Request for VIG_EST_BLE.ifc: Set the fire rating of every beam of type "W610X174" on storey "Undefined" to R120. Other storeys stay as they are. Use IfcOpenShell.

First a look at what the model holds.

```python
import ifcopenshell
import ifcopenshell.util.element

model = ifcopenshell.open("VIG_EST_BLE.ifc")
print(model.schema)
storey = next(s for s in model.by_type("IfcBuildingStorey") if s.Name == "Undefined")
beams = [e for e in ifcopenshell.util.element.get_decomposition(storey) if e.is_a("IfcBeam")]
seen = {}
for e in beams:
    element_type = ifcopenshell.util.element.get_type(e)
    key = (element_type.Name if element_type != e and element_type else None, ifcopenshell.util.element.get_pset(e, "Pset_BeamCommon", "FireRating"))
    seen[key] = seen.get(key, 0) + 1
for (name, value), count in sorted(seen.items(), key=str):
    print(count, "x", name, "|", value)
```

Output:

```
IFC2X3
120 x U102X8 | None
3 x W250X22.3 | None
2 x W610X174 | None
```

```python
import ifcopenshell
import ifcopenshell.api.pset
import ifcopenshell.util.element

model = ifcopenshell.open("VIG_EST_BLE.ifc")

storey = next(s for s in model.by_type("IfcBuildingStorey") if s.Name == "Undefined")
beams = [e for e in ifcopenshell.util.element.get_decomposition(storey) if e.is_a("IfcBeam")]

count = 0
for e in beams:
    element_type = ifcopenshell.util.element.get_type(e)
    if element_type in (None, e) or element_type.Name != "W610X174":
        continue
    found = ifcopenshell.util.element.get_pset(e, "Pset_BeamCommon", should_inherit=False)
    if found:
        pset = model.by_id(found["id"])
        if len(ifcopenshell.util.element.get_elements_by_pset(pset)) > 1:
            pset = ifcopenshell.api.pset.unshare_pset(model, products=[e], pset=pset)[0]
    else:
        pset = ifcopenshell.api.pset.add_pset(model, product=e, name="Pset_BeamCommon")
    ifcopenshell.api.pset.edit_pset(model, pset=pset, properties={"FireRating": "R120"})
    count += 1

print(count, "beams updated")

model.write("VIG_EST_BLE_rev.ifc")
```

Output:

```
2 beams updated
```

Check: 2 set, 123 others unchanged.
